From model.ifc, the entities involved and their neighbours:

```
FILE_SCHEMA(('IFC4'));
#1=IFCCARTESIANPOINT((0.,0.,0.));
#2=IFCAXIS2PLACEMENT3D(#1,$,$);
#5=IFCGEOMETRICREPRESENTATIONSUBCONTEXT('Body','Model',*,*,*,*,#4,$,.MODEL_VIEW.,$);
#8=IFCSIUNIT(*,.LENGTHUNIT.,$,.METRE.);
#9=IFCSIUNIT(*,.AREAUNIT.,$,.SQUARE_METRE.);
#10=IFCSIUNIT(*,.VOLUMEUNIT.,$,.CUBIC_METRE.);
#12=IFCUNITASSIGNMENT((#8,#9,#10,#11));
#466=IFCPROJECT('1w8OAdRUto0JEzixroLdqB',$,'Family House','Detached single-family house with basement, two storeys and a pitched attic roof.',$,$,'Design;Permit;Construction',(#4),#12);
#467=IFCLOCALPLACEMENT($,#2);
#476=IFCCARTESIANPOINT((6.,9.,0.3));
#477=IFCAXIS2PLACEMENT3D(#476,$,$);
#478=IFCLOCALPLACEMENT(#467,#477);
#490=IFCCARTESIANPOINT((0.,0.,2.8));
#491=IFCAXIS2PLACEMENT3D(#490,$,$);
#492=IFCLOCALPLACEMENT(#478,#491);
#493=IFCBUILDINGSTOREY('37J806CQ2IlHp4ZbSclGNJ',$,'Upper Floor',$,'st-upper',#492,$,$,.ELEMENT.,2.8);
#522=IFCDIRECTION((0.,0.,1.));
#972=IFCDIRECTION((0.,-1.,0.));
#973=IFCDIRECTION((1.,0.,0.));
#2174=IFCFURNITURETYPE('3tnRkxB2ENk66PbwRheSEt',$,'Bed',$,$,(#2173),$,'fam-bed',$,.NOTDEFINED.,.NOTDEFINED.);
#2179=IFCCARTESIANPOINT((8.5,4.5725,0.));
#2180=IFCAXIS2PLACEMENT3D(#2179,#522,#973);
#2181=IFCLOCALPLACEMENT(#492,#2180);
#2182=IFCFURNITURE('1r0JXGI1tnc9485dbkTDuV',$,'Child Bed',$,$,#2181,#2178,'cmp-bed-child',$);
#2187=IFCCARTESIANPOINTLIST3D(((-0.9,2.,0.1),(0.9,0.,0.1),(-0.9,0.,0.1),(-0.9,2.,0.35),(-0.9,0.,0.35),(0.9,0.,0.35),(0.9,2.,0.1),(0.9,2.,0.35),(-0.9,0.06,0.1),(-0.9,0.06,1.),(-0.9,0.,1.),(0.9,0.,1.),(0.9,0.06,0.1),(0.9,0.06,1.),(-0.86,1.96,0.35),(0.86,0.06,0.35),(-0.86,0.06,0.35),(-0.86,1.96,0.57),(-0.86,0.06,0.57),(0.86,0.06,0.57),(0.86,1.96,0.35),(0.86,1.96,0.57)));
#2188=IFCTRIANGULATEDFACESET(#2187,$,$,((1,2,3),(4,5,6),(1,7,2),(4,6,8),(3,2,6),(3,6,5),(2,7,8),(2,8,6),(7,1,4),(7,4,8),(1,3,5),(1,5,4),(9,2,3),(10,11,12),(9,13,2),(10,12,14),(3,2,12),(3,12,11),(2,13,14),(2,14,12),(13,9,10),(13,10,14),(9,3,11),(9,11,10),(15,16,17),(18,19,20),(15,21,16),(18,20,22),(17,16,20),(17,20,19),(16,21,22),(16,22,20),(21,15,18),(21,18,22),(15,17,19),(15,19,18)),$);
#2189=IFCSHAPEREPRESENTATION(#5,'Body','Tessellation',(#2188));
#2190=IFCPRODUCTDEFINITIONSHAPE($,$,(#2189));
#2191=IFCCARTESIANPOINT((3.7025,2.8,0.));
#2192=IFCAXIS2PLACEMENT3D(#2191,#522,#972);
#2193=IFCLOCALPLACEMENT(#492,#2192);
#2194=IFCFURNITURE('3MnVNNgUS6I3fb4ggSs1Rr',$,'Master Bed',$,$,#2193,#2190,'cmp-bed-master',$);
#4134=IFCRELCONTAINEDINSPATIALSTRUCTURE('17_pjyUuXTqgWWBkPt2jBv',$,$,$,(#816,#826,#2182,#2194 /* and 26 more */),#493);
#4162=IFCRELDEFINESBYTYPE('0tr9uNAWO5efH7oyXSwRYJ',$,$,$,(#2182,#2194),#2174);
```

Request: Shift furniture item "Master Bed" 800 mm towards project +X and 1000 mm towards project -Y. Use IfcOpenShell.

```python
import ifcopenshell
import ifcopenshell.api.geometry
import ifcopenshell.util.placement

model = ifcopenshell.open("model.ifc")

item = model.by_guid("3MnVNNgUS6I3fb4ggSs1Rr")
matrix = ifcopenshell.util.placement.get_local_placement(item.ObjectPlacement)
matrix[0, 3] += 0.8
matrix[1, 3] -= 1.0
ifcopenshell.api.geometry.edit_object_placement(model, product=item, matrix=matrix, is_si=False)

print(ifcopenshell.util.placement.get_local_placement(item.ObjectPlacement).round(3) + 0.0)

model.write("model_v2.ifc")
```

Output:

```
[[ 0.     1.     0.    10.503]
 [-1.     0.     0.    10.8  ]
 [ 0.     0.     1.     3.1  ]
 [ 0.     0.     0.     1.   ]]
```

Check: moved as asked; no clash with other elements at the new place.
